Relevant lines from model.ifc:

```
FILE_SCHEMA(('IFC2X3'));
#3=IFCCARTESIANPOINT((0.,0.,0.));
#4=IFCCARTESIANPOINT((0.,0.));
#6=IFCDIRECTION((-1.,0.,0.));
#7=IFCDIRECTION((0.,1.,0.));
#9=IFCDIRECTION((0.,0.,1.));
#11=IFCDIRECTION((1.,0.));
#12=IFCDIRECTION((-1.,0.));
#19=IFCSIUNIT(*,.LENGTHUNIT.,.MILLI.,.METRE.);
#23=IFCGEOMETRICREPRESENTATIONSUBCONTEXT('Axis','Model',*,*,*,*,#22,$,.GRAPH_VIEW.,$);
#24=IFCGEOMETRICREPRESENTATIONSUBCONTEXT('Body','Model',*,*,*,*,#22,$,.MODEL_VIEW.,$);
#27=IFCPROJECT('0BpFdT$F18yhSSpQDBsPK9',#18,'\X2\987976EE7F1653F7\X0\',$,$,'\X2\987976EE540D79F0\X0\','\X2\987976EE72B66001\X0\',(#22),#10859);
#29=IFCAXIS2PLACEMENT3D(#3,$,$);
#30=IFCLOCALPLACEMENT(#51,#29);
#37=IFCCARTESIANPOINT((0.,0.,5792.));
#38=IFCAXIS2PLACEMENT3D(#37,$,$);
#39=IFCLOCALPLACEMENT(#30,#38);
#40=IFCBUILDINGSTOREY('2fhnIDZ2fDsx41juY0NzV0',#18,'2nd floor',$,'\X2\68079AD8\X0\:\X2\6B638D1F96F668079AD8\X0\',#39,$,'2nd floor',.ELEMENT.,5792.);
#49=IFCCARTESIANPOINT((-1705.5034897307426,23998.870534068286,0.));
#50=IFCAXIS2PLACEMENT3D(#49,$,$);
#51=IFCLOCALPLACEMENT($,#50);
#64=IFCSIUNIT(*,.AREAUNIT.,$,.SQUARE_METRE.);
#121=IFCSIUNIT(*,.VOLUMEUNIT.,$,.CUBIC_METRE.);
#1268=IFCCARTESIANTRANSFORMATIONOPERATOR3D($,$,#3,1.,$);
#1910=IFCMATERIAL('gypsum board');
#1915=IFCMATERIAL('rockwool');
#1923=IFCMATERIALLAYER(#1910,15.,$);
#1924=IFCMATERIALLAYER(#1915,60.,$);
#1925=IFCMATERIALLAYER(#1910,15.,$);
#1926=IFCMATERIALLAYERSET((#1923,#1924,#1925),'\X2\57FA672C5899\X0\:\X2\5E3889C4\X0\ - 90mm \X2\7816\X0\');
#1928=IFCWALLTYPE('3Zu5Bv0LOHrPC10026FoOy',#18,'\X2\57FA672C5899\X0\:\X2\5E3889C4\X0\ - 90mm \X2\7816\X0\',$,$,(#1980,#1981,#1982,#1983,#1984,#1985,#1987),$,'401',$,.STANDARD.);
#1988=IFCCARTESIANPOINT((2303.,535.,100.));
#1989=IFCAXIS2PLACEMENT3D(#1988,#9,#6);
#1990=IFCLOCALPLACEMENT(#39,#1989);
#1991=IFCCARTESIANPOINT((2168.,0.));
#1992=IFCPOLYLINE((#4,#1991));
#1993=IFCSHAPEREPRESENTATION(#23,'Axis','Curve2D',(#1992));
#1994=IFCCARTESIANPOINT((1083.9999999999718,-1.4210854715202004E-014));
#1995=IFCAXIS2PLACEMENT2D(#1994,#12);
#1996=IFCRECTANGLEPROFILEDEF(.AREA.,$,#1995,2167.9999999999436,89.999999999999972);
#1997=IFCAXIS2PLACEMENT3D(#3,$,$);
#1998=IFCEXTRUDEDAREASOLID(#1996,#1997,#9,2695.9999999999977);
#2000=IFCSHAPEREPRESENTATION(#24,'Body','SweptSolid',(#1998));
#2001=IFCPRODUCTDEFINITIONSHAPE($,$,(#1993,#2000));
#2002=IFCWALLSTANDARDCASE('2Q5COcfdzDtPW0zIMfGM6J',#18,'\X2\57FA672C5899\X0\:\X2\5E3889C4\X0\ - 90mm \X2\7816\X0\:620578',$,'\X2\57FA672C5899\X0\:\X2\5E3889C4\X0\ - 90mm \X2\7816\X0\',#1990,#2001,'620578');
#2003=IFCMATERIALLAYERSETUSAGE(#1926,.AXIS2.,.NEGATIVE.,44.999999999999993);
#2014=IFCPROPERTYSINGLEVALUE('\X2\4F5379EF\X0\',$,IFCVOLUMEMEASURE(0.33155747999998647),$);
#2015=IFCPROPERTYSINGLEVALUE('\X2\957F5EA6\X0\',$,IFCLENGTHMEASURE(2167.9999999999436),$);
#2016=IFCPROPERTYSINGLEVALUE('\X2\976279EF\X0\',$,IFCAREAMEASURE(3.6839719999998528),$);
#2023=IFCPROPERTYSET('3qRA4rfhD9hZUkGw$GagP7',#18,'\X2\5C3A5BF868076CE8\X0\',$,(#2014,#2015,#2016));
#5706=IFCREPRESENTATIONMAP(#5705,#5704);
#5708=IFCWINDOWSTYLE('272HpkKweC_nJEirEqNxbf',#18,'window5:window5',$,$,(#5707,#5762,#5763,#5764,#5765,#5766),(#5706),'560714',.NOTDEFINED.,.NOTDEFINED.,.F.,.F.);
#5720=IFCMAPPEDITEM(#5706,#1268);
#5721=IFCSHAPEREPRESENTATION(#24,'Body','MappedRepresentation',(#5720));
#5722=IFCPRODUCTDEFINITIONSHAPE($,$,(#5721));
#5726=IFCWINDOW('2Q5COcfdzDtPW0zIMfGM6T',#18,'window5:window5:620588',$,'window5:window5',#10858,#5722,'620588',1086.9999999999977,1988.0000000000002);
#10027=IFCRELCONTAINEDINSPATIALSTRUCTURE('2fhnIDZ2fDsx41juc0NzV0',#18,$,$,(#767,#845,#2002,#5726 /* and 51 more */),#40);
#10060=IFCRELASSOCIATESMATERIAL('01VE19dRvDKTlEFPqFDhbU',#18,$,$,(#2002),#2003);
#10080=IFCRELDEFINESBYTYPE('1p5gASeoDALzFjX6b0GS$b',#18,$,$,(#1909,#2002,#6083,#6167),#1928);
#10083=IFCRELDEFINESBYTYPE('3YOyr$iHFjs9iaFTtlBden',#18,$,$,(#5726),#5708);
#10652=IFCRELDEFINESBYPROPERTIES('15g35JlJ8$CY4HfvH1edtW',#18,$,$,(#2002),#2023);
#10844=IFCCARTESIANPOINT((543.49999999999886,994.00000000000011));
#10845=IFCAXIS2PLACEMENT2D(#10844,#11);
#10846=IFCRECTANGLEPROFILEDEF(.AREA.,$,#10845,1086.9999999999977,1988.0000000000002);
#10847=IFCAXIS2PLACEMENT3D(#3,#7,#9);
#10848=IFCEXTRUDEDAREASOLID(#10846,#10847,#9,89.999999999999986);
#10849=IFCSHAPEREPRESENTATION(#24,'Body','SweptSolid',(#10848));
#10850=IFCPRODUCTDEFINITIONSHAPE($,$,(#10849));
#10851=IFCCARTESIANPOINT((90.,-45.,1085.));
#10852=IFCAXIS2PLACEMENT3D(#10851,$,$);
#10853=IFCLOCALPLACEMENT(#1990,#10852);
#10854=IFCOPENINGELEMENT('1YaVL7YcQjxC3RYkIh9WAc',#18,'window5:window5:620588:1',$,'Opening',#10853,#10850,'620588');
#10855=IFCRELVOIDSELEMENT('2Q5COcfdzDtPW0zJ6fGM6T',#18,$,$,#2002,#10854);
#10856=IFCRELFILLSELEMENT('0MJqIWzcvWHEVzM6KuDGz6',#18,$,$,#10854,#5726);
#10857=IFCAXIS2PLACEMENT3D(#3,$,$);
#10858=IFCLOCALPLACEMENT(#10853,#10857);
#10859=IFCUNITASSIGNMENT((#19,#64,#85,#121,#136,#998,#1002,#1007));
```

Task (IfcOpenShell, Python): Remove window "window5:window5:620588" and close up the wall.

```python
import ifcopenshell
import ifcopenshell.api.feature
import ifcopenshell.api.pset
import ifcopenshell.api.root
import ifcopenshell.geom
import ifcopenshell.util.element
import ifcopenshell.util.shape
import ifcopenshell.util.unit

model = ifcopenshell.open("model.ifc")
area_scale = ifcopenshell.util.unit.calculate_unit_scale(model, "AREAUNIT")
volume_scale = ifcopenshell.util.unit.calculate_unit_scale(model, "VOLUMEUNIT")
settings = ifcopenshell.geom.settings()


def volume(element):
    """Net volume in cubic metres, openings subtracted."""
    shape = ifcopenshell.geom.create_shape(settings, element)
    return ifcopenshell.util.shape.get_volume(shape.geometry)


window = model.by_guid("2Q5COcfdzDtPW0zIMfGM6T")
opening = window.FillsVoids[0].RelatingOpeningElement
wall = opening.VoidsElements[0].RelatingBuildingElement
before = volume(wall)

ifcopenshell.api.root.remove_product(model, product=window)
ifcopenshell.api.feature.remove_feature(model, feature=opening)

after = volume(wall)
thickness = 0.09  # wall thickness in metres

# Update the wall's stored quantities.
pset = model.by_id(ifcopenshell.util.element.get_pset(wall, "尺寸标注", should_inherit=False)["id"])
ifcopenshell.api.pset.edit_pset(model, pset=pset, properties={
    "体积": model.create_entity("IfcVolumeMeasure", after / volume_scale),
    "面积": model.create_entity("IfcAreaMeasure", after / thickness / area_scale),
})

print(f"wall volume {before:.3f} -> {after:.3f} m3")

model.write("model_edited.ifc")
```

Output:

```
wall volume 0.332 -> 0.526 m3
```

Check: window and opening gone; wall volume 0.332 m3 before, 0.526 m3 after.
